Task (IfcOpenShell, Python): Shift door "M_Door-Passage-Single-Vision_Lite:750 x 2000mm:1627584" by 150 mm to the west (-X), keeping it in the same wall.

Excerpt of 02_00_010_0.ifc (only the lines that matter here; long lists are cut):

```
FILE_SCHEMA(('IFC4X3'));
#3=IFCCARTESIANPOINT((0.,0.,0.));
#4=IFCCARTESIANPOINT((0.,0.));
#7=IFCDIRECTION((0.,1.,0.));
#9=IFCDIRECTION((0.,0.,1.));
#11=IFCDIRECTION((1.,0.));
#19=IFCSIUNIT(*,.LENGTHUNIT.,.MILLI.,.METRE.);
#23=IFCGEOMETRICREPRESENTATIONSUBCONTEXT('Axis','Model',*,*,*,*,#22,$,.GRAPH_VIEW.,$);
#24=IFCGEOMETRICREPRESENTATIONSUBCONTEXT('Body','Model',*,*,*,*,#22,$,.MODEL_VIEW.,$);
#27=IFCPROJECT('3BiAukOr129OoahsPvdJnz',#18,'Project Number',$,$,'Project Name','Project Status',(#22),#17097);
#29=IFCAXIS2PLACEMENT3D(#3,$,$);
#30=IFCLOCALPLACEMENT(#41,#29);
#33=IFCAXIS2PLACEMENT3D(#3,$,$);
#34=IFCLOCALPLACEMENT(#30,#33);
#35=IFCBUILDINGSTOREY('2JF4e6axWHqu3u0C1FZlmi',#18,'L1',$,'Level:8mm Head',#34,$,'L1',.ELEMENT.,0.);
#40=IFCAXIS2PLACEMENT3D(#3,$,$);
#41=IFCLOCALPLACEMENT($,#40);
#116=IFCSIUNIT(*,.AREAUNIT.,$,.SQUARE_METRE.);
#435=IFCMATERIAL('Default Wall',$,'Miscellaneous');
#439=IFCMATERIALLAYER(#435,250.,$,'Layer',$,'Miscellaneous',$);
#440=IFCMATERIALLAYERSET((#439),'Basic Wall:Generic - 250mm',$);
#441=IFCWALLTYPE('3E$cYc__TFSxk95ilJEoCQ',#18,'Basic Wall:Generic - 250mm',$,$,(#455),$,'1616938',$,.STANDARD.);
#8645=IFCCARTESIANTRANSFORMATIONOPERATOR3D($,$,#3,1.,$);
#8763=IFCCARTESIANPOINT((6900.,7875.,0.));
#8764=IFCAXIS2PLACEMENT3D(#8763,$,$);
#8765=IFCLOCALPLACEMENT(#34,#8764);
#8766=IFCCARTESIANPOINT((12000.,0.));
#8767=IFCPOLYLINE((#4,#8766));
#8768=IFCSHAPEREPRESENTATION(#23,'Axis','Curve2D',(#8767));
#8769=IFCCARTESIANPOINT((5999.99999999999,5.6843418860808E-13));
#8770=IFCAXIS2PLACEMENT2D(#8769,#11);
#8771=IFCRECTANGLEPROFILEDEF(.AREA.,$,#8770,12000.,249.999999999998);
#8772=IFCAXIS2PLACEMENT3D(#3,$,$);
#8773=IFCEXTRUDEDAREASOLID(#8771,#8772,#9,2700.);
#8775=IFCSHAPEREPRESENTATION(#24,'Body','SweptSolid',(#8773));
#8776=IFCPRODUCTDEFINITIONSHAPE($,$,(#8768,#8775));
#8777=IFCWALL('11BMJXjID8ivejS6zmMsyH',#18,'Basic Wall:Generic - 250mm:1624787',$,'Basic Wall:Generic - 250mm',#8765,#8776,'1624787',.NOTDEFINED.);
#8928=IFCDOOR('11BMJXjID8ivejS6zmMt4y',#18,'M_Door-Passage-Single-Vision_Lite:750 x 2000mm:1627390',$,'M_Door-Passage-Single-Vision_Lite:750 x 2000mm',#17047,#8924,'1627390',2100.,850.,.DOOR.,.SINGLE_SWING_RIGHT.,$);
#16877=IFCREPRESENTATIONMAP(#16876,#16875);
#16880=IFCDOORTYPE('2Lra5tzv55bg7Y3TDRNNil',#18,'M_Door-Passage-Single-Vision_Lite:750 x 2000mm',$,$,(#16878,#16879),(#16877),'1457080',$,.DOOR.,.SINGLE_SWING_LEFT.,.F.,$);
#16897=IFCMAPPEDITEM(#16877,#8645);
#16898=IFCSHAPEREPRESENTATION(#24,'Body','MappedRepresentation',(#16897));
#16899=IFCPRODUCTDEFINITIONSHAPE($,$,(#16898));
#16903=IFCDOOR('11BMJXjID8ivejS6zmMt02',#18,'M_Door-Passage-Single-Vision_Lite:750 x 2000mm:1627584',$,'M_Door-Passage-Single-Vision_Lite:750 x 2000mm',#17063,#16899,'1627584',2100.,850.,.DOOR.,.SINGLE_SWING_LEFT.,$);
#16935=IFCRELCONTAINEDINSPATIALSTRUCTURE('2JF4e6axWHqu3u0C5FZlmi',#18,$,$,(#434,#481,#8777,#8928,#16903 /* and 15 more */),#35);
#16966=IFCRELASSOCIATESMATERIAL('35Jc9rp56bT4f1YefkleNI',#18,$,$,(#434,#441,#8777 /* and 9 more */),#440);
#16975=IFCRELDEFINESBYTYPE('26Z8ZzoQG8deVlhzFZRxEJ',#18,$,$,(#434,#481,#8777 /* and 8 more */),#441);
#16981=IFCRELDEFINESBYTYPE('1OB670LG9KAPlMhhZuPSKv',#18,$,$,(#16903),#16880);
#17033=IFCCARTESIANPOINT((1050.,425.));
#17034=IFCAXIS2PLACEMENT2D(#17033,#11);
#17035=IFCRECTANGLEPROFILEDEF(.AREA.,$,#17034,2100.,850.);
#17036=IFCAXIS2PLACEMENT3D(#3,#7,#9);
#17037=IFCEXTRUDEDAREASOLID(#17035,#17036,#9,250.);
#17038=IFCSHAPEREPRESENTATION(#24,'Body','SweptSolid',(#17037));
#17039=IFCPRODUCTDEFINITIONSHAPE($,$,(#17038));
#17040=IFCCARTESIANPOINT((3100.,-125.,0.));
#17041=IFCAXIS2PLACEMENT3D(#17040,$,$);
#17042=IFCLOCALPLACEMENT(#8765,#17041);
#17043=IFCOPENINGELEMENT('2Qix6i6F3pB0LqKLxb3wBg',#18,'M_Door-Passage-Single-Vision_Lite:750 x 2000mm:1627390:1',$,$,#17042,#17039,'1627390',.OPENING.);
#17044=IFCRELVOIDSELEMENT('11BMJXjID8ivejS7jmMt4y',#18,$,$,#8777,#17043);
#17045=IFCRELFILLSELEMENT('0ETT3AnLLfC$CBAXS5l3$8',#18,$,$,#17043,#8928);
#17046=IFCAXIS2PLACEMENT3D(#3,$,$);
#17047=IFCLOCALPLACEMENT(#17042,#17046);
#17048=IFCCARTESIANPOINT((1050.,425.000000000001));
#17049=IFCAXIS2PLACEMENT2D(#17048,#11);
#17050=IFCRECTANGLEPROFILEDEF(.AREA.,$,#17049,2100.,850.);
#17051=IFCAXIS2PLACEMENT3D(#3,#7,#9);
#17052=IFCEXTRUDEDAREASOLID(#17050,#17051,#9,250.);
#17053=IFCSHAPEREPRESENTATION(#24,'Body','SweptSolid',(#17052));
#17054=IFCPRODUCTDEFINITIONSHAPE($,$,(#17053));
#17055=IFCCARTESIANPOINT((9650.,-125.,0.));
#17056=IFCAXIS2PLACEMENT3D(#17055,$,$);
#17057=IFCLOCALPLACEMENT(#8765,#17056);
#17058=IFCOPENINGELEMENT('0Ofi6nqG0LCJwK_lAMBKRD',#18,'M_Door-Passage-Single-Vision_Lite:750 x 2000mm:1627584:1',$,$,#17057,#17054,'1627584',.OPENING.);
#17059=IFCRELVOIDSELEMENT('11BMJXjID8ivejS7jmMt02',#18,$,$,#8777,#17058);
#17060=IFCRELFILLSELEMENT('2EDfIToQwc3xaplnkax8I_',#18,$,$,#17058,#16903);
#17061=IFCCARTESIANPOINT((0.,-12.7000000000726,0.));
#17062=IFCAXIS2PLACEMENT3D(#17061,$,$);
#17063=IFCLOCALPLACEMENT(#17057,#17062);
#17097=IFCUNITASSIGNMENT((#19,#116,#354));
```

```python
import ifcopenshell
import ifcopenshell.api.geometry
import ifcopenshell.util.placement

model = ifcopenshell.open("02_00_010_0.ifc")

door = model.by_id(16903)
opening = door.FillsVoids[0].RelatingOpeningElement
wall = opening.VoidsElements[0].RelatingBuildingElement

wall_matrix = ifcopenshell.util.placement.get_local_placement(wall.ObjectPlacement)
shift = wall_matrix[:3, 0] * -150.0
before = ifcopenshell.util.placement.get_local_placement(door.ObjectPlacement)[:3, 3].copy()

# The door is placed relative to its opening, so it follows when the opening moves.
matrix = ifcopenshell.util.placement.get_local_placement(opening.ObjectPlacement)
matrix[:3, 3] += shift
ifcopenshell.api.geometry.edit_object_placement(
    model, product=opening, matrix=matrix, is_si=False, should_transform_children=True
)

after = ifcopenshell.util.placement.get_local_placement(door.ObjectPlacement)[:3, 3]
print("door moved by", (after - before).round(3) + 0.0)

model.write("02_00_010_0_updated.ifc")
```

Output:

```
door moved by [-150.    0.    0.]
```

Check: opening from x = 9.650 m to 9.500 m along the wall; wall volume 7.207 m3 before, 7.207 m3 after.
